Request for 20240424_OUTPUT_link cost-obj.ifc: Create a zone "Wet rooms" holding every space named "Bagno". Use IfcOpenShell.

First a look at what the model holds.

```python
import ifcopenshell

model = ifcopenshell.open("20240424_OUTPUT_link cost-obj.ifc")
print(model.schema)
seen = {}
for space in model.by_type("IfcSpace"):
    seen[space.LongName] = seen.get(space.LongName, 0) + 1
for name, count in sorted(seen.items(), key=str):
    print(count, "x", name)
print("zones:", [z.Name for z in model.by_type("IfcZone")][:20])
```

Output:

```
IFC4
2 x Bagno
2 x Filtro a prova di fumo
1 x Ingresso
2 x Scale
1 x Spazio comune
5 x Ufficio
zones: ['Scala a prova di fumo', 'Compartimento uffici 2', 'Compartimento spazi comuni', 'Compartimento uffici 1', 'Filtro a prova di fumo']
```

```python
import ifcopenshell
import ifcopenshell.api.group
import ifcopenshell.api.root

model = ifcopenshell.open("20240424_OUTPUT_link cost-obj.ifc")

names = {"Bagno"}
spaces = [s for s in model.by_type("IfcSpace") if s.LongName in names]

zone = ifcopenshell.api.root.create_entity(model, ifc_class="IfcZone", name="Wet rooms")
ifcopenshell.api.group.assign_group(model, products=spaces, group=zone)
print(len(spaces), "spaces in", zone.Name)

model.write("20240424_OUTPUT_link cost-obj_updated.ifc")
```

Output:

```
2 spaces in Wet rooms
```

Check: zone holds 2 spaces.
